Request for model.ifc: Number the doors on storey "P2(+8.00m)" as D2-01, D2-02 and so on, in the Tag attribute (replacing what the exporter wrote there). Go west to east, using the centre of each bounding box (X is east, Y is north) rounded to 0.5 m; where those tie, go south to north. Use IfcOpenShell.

First a look at what the model holds.

```python
import ifcopenshell
import ifcopenshell.util.element
import ifcopenshell.util.placement

model = ifcopenshell.open("model.ifc")
print(model.schema)
storey = next(s for s in model.by_type("IfcBuildingStorey") if s.Name == "P2(+8.00m)")
doors = [e for e in ifcopenshell.util.element.get_decomposition(storey) if e.is_a("IfcDoor")]
for e in sorted(doors, key=lambda e: e.id()):
    origin = ifcopenshell.util.placement.get_local_placement(e.ObjectPlacement)[:3, 3]
    print(e.id(), e.Tag, e.Name, origin.round(2) + 0.0, sep=" | ")
```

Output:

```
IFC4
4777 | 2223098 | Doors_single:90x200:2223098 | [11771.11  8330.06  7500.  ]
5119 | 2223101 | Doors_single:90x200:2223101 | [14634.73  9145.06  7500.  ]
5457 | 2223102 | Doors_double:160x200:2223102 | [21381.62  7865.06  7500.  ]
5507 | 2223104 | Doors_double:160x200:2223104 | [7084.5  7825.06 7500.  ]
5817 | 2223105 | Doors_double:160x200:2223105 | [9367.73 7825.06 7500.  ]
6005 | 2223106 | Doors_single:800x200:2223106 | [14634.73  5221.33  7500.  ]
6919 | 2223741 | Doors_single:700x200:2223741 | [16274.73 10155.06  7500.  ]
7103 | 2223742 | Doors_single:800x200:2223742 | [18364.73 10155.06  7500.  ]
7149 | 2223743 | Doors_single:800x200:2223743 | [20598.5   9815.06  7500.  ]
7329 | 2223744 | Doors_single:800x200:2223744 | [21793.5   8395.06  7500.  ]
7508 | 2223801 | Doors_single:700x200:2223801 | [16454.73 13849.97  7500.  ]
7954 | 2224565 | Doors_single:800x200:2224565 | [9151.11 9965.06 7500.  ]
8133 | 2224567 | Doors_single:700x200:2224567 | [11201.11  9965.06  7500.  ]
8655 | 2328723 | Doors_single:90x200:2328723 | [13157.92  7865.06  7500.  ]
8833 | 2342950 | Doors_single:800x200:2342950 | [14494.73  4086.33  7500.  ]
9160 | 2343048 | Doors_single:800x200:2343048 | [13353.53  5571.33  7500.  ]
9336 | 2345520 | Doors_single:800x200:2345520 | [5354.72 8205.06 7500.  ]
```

```python
import ifcopenshell
import ifcopenshell.geom
import ifcopenshell.util.element
import ifcopenshell.util.shape

model = ifcopenshell.open("model.ifc")
settings = ifcopenshell.geom.settings()
settings.set("use-world-coords", True)


def centre(element):
    shape = ifcopenshell.geom.create_shape(settings, element)
    return ifcopenshell.util.shape.get_bbox_centroid(shape.geometry)


storey = next(s for s in model.by_type("IfcBuildingStorey") if s.Name == "P2(+8.00m)")
doors = [e for e in ifcopenshell.util.element.get_decomposition(storey) if e.is_a("IfcDoor")]

# Insertion points can sit at a corner or the storey origin, so sort by the geometry (in metres).
centres = {e: centre(e) for e in doors}
doors.sort(key=lambda e: (round(centres[e][0] / 0.5), centres[e][1]))

for i, e in enumerate(doors, start=1):
    number = f"D2-{i:02d}"
    e.Tag = number
    print(e.id(), number)

model.write("model_rev.ifc")
```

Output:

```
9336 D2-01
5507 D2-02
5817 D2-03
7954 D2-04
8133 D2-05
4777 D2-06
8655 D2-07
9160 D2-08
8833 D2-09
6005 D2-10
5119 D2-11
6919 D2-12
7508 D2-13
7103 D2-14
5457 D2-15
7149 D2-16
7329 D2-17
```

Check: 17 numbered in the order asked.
